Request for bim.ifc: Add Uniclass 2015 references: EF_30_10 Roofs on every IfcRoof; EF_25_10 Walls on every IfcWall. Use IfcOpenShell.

First a look at what the model holds.

```python
import ifcopenshell

model = ifcopenshell.open("bim.ifc")
print(model.schema)
print("classifications:", [c.Name for c in model.by_type("IfcClassification")])
for ifc_class in ("IfcDoor", "IfcRoof", "IfcStair", "IfcWall", "IfcWindow"):
    print(ifc_class, len(model.by_type(ifc_class)))
```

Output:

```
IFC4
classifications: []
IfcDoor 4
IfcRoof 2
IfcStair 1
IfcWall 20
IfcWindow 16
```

```python
import ifcopenshell
import ifcopenshell.api.classification

model = ifcopenshell.open("bim.ifc")

system = ifcopenshell.api.classification.add_classification(model, classification="Uniclass 2015")

codes = {
    "IfcRoof": ("EF_30_10", "Roofs"),
    "IfcWall": ("EF_25_10", "Walls"),
}
for ifc_class, (code, name) in codes.items():
    products = model.by_type(ifc_class)
    ifcopenshell.api.classification.add_reference(
        model, products=products, classification=system, identification=code, name=name
    )
    print(code, len(products))

model.write("bim_rev.ifc")
```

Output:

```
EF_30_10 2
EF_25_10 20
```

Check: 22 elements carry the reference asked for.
